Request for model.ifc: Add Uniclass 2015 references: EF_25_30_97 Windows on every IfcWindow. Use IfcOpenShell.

First a look at what the model holds.

```python
import ifcopenshell

model = ifcopenshell.open("model.ifc")
print(model.schema)
print("classifications:", [c.Name for c in model.by_type("IfcClassification")])
for ifc_class in ("IfcDoor", "IfcRoof", "IfcStair", "IfcWall", "IfcWindow"):
    print(ifc_class, len(model.by_type(ifc_class)))
```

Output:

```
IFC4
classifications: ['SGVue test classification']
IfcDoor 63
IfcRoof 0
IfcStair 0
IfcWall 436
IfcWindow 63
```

```python
import ifcopenshell
import ifcopenshell.api.classification

model = ifcopenshell.open("model.ifc")

system = ifcopenshell.api.classification.add_classification(model, classification="Uniclass 2015")

codes = {
    "IfcWindow": ("EF_25_30_97", "Windows"),
}
for ifc_class, (code, name) in codes.items():
    products = model.by_type(ifc_class)
    ifcopenshell.api.classification.add_reference(
        model, products=products, classification=system, identification=code, name=name
    )
    print(code, len(products))

model.write("model_edited.ifc")
```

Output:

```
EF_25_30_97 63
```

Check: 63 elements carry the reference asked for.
